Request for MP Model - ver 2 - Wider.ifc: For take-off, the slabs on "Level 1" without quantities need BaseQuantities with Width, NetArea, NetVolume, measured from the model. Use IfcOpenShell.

First a look at what the model holds.

```python
import ifcopenshell
import ifcopenshell.util.element
import ifcopenshell.util.unit

model = ifcopenshell.open("MP Model - ver 2 - Wider.ifc")
print(model.schema)
for unit_type in ("LENGTHUNIT", "AREAUNIT", "VOLUMEUNIT"):
    print(unit_type, ifcopenshell.util.unit.calculate_unit_scale(model, unit_type))
storey = next(s for s in model.by_type("IfcBuildingStorey") if s.Name == "Level 1")
slabs = [e for e in ifcopenshell.util.element.get_decomposition(storey) if e.is_a("IfcSlab")]
for e in sorted(slabs, key=lambda e: e.id()):
    print(e.id(), e.is_a(), e.Name, list(ifcopenshell.util.element.get_psets(e, qtos_only=True)), sep=" | ")
```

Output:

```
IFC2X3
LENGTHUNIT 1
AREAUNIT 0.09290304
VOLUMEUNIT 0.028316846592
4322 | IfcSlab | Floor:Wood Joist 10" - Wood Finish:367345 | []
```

```python
import ifcopenshell
import ifcopenshell.api.pset
import ifcopenshell.geom
import ifcopenshell.util.element
import ifcopenshell.util.shape
import ifcopenshell.util.unit

model = ifcopenshell.open("MP Model - ver 2 - Wider.ifc")
unit_scale = ifcopenshell.util.unit.calculate_unit_scale(model)
area_scale = ifcopenshell.util.unit.calculate_unit_scale(model, "AREAUNIT")
volume_scale = ifcopenshell.util.unit.calculate_unit_scale(model, "VOLUMEUNIT")
settings = ifcopenshell.geom.settings()

storey = next(s for s in model.by_type("IfcBuildingStorey") if s.Name == "Level 1")
slabs = [e for e in ifcopenshell.util.element.get_decomposition(storey) if e.is_a("IfcSlab")]

for e in sorted(slabs, key=lambda e: e.id()):
    if ifcopenshell.util.element.get_psets(e, qtos_only=True, should_inherit=False):
        continue
    # Geometry comes back in metres, in the element's own axes.
    shape = ifcopenshell.geom.create_shape(settings, e)
    values = {
        "Width": ifcopenshell.util.shape.get_z(shape.geometry) / unit_scale,
        "NetArea": ifcopenshell.util.shape.get_footprint_area(shape.geometry) / area_scale,
        "NetVolume": ifcopenshell.util.shape.get_volume(shape.geometry) / volume_scale,
    }
    qto = ifcopenshell.api.pset.add_qto(model, product=e, name="BaseQuantities")
    ifcopenshell.api.pset.edit_qto(model, qto=qto, properties=values)
    print(e.id(), {k: round(v, 3) for k, v in values.items()})

model.write("MP Model - ver 2 - Wider_updated.ifc")
```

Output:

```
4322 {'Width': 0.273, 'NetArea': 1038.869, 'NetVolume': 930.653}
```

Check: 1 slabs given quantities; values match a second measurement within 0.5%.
